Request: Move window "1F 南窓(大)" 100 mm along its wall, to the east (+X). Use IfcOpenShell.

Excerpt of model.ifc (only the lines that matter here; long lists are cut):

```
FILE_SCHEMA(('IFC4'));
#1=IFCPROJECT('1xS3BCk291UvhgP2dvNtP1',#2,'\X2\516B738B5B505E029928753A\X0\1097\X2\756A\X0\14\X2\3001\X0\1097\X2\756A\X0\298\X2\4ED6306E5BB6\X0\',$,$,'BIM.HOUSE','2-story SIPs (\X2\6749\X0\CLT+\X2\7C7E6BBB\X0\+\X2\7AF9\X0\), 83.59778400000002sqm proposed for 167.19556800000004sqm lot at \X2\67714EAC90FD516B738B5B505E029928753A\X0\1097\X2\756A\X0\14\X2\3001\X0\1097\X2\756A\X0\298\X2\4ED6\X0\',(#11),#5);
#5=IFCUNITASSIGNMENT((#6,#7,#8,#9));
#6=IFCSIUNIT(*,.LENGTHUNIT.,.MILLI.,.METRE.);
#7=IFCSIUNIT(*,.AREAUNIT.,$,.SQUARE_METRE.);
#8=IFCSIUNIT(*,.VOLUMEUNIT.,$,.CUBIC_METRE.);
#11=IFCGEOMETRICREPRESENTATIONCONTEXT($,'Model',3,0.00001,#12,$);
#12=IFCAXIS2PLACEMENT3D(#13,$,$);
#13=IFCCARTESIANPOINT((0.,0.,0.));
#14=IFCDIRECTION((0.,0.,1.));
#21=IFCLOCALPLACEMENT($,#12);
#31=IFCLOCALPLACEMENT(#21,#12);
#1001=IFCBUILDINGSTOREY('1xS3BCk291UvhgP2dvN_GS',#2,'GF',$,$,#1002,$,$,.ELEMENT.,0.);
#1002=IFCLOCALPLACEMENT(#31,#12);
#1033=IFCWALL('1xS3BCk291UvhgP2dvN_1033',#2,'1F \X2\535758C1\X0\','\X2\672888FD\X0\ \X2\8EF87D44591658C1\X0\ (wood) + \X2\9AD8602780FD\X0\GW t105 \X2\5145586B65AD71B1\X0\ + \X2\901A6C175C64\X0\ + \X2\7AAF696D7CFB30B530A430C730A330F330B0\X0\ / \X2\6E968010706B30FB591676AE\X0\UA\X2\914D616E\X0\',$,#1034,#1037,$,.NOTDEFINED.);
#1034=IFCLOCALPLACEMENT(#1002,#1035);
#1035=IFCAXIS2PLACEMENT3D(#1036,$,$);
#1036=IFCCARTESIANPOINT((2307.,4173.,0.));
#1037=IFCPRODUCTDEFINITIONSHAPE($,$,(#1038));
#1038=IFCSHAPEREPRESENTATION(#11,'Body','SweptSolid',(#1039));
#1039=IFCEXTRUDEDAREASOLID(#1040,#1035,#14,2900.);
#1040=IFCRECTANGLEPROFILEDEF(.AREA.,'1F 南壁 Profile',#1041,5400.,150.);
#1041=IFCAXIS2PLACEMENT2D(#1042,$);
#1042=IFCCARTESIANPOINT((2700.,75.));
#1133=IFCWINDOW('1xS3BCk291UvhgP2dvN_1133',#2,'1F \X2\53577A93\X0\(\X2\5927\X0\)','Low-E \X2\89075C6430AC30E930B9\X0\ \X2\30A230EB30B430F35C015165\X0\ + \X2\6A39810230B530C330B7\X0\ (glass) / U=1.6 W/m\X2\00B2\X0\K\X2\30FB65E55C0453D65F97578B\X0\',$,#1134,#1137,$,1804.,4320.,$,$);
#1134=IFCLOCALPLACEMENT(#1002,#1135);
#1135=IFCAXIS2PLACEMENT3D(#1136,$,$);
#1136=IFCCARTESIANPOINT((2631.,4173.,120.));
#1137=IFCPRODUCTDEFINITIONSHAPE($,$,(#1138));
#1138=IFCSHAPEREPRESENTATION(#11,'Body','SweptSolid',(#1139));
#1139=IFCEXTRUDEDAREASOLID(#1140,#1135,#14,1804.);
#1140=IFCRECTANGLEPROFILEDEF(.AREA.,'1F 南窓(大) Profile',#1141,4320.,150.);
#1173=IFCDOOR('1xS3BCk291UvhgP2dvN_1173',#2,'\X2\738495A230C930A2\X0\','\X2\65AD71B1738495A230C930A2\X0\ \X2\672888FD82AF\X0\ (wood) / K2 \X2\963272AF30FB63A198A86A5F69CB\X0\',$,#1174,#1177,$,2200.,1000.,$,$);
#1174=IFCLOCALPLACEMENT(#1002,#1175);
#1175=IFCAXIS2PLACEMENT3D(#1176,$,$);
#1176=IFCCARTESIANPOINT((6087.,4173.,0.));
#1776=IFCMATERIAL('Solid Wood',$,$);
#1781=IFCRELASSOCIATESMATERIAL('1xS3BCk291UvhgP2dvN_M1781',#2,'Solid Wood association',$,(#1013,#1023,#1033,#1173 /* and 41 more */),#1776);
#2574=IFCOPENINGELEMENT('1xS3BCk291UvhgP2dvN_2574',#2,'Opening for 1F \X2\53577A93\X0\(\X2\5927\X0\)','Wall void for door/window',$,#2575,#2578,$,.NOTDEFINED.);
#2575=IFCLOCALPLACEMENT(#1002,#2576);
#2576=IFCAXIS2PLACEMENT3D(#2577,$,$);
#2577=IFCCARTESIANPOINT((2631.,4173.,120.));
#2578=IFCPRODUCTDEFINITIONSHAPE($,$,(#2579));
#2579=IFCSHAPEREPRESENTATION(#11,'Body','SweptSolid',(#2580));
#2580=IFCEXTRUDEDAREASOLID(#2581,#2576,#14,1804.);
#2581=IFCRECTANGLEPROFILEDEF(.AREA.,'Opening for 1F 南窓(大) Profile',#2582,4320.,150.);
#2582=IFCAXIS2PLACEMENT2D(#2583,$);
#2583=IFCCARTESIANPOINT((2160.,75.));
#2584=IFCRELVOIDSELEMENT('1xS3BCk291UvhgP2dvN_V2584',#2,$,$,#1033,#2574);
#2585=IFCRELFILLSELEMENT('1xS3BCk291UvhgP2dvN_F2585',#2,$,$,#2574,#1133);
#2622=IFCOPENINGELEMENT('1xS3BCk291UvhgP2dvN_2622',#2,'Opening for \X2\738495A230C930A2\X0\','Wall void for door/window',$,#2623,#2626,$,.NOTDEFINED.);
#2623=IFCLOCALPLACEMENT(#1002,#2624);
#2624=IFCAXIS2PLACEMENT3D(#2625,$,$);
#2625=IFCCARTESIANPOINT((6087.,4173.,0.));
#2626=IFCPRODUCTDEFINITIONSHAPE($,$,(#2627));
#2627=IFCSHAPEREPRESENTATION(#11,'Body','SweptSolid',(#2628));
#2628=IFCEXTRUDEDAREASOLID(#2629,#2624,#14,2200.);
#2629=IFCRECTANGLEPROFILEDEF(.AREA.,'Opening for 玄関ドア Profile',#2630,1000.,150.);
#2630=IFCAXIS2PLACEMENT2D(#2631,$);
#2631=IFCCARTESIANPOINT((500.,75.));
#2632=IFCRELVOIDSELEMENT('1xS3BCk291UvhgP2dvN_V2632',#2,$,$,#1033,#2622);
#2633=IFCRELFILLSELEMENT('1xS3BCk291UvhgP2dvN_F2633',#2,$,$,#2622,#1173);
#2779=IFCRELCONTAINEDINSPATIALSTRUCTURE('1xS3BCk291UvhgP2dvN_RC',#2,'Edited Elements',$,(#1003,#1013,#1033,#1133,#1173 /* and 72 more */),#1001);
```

```python
import ifcopenshell
import ifcopenshell.api.geometry
import ifcopenshell.util.placement
import ifcopenshell.util.unit

model = ifcopenshell.open("model.ifc")
unit_scale = ifcopenshell.util.unit.calculate_unit_scale(model)

window = model.by_guid("1xS3BCk291UvhgP2dvN_1133")
opening = window.FillsVoids[0].RelatingOpeningElement
wall = opening.VoidsElements[0].RelatingBuildingElement

wall_matrix = ifcopenshell.util.placement.get_local_placement(wall.ObjectPlacement)
shift = wall_matrix[:3, 0] * 0.1 / unit_scale
before = ifcopenshell.util.placement.get_local_placement(window.ObjectPlacement)[:3, 3].copy()

# The window is not placed relative to its opening, so move both.
for product in (opening, window):
    matrix = ifcopenshell.util.placement.get_local_placement(product.ObjectPlacement)
    matrix[:3, 3] += shift
    ifcopenshell.api.geometry.edit_object_placement(model, product=product, matrix=matrix, is_si=False)

after = ifcopenshell.util.placement.get_local_placement(window.ObjectPlacement)[:3, 3]
print("window moved by", (after - before).round(3) + 0.0)

model.write("model-out.ifc")
```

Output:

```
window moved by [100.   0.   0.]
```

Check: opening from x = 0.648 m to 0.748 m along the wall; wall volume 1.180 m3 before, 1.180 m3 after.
